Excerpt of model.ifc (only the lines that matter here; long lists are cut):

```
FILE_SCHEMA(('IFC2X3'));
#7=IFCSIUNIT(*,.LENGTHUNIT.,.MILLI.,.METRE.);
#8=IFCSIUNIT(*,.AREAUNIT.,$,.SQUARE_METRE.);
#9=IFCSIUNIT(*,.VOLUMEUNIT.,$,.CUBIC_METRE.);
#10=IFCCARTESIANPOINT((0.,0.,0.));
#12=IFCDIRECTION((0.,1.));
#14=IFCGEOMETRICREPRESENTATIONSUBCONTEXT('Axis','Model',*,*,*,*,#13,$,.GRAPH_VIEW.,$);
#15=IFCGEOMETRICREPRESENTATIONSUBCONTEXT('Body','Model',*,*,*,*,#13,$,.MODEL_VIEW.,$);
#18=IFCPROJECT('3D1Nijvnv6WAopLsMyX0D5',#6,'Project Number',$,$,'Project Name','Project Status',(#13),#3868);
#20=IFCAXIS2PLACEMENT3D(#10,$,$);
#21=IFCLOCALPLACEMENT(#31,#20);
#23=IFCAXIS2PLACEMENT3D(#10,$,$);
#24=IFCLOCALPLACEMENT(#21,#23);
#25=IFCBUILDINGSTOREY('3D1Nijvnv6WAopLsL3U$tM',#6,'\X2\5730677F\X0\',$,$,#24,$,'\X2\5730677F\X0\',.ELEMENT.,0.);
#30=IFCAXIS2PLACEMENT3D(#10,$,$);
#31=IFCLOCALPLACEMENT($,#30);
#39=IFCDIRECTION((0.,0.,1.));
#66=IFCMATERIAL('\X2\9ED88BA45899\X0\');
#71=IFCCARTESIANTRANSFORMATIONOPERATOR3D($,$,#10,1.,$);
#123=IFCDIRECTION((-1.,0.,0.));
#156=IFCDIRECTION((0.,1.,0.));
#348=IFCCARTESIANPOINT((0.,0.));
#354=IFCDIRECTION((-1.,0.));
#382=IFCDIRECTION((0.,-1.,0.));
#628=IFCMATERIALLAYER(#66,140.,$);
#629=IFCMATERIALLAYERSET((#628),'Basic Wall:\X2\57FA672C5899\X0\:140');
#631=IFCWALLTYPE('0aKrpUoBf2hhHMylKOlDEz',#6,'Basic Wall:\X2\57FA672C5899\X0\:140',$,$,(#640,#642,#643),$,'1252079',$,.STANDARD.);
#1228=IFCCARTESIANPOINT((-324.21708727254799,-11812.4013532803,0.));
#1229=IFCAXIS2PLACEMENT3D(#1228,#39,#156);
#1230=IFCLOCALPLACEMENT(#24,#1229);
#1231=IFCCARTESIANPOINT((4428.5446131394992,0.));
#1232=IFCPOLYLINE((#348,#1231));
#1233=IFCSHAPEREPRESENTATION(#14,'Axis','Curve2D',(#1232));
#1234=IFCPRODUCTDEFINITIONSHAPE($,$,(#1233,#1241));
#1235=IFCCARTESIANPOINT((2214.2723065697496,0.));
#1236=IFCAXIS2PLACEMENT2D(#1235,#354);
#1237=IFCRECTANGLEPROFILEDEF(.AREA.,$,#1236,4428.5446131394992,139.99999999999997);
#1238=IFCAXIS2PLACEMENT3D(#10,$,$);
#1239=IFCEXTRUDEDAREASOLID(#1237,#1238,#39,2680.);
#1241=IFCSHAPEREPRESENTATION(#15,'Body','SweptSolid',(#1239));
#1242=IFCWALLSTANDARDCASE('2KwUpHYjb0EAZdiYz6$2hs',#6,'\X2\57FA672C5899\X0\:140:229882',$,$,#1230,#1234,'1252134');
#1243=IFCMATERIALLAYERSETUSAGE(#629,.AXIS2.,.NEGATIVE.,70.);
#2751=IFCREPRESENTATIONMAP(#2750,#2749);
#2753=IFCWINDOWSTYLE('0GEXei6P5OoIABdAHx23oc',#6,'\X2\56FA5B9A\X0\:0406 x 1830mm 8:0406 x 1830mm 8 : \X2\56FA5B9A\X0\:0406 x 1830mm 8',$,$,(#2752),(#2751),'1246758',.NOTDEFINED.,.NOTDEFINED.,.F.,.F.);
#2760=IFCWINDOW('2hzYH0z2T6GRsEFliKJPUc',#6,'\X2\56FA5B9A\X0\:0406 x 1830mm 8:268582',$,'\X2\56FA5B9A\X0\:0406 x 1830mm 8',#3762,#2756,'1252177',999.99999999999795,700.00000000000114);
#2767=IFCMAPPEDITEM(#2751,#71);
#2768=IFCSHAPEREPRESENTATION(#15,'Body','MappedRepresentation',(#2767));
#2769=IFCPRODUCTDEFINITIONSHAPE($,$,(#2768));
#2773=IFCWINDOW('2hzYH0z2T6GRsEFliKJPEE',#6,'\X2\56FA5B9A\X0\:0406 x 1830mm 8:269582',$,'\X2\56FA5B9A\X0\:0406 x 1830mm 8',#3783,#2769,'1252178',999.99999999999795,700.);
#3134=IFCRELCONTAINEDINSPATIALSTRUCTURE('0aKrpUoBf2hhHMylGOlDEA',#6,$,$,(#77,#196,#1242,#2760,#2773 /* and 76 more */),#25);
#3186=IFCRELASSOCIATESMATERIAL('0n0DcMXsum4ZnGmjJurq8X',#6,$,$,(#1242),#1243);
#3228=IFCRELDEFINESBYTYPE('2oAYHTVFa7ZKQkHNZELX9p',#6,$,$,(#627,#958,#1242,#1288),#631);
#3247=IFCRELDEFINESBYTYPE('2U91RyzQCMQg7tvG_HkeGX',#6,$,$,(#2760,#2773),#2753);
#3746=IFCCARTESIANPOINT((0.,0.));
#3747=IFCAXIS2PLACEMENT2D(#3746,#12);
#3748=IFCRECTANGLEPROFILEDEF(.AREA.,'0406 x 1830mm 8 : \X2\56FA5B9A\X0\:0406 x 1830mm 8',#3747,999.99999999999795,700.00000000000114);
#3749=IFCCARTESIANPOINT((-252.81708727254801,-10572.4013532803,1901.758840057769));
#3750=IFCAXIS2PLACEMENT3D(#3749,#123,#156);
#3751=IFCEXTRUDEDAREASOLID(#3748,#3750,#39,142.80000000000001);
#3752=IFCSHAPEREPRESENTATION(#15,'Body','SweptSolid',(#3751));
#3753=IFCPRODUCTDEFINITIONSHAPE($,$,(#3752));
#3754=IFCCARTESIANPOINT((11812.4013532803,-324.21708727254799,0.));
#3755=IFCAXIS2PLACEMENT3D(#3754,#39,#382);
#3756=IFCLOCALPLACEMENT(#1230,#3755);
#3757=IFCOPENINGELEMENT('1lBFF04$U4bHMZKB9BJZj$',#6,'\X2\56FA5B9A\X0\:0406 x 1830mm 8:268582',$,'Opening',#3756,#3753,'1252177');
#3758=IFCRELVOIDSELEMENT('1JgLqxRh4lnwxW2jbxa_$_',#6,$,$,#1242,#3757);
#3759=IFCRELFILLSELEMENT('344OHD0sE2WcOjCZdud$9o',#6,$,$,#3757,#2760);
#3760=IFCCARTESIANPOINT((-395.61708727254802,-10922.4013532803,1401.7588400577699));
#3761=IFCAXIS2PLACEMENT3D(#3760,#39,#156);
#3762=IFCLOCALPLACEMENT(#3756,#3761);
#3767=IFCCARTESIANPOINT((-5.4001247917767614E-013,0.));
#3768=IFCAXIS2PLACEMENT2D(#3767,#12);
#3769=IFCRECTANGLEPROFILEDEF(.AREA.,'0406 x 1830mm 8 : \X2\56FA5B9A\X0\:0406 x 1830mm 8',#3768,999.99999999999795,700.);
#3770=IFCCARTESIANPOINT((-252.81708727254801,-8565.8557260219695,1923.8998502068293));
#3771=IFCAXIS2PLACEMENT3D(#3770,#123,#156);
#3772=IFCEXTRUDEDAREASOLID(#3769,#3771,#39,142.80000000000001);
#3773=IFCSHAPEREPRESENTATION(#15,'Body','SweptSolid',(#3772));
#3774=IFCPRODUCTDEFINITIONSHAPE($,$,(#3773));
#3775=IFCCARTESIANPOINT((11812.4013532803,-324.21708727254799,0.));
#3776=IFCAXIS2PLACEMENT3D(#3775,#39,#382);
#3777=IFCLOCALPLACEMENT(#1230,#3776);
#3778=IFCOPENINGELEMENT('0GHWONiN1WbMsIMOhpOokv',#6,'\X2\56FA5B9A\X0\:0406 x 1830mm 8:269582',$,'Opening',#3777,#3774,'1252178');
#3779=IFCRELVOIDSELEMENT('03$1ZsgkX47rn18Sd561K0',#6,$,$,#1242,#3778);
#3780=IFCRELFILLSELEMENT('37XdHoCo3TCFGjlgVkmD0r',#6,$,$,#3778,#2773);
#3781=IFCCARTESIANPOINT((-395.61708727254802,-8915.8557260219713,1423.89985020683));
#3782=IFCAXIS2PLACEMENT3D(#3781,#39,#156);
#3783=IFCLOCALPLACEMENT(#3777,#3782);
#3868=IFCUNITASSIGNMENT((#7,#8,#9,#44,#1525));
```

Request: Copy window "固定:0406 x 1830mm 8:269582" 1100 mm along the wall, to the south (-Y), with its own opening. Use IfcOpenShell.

```python
import ifcopenshell
import ifcopenshell.api.feature
import ifcopenshell.api.geometry
import ifcopenshell.api.root
import ifcopenshell.geom
import ifcopenshell.util.element
import ifcopenshell.util.placement
import ifcopenshell.util.shape
import ifcopenshell.util.unit

model = ifcopenshell.open("model.ifc")
unit_scale = ifcopenshell.util.unit.calculate_unit_scale(model)
settings = ifcopenshell.geom.settings()


def volume(element):
    """Net volume in cubic metres, openings subtracted."""
    shape = ifcopenshell.geom.create_shape(settings, element)
    return ifcopenshell.util.shape.get_volume(shape.geometry)


def reuse_history(source, copy):
    """copy_class also copies each property set's owner history, people and application; keep the originals."""
    for rel in copy.IsDefinedBy:
        if rel.is_a("IfcRelDefinesByProperties") and (history := rel.RelatingPropertyDefinition.OwnerHistory):
            rel.RelatingPropertyDefinition.OwnerHistory = source.OwnerHistory
            ifcopenshell.util.element.remove_deep2(model, history)


window = model.by_guid("2hzYH0z2T6GRsEFliKJPEE")
opening = window.FillsVoids[0].RelatingOpeningElement
wall = opening.VoidsElements[0].RelatingBuildingElement
before = volume(wall)
shift = ifcopenshell.util.placement.get_local_placement(wall.ObjectPlacement)[:3, 0] * -1.1 / unit_scale

# copy_class copies the void relationship, type, container and properties, but no geometry.
new_opening = ifcopenshell.api.root.copy_class(model, product=opening)
new_opening.Representation = ifcopenshell.util.element.copy_deep(
    model, opening.Representation, exclude=["IfcGeometricRepresentationContext", "IfcRepresentationMap"]
)
new_opening.Name = "固定:0406 x 1830mm 8"
new_opening.Tag = None
new_window = ifcopenshell.api.root.copy_class(model, product=window)
new_window.Representation = ifcopenshell.util.element.copy_deep(
    model, window.Representation, exclude=["IfcGeometricRepresentationContext", "IfcRepresentationMap"]
)
new_window.Name = "固定:0406 x 1830mm 8"
new_window.Tag = None
reuse_history(window, new_window)
fills = ifcopenshell.api.feature.add_filling(model, opening=new_opening, element=new_window)
fills.OwnerHistory = new_window.OwnerHistory  # required in IFC2X3

for old, new in ((opening, new_opening), (window, new_window)):
    matrix = ifcopenshell.util.placement.get_local_placement(old.ObjectPlacement)
    matrix[:3, 3] += shift
    ifcopenshell.api.geometry.edit_object_placement(model, product=new, matrix=matrix, is_si=False)

after = volume(wall)

print(f"wall volume {before:.3f} -> {after:.3f} m3")

model.write("model_edited.ifc")
```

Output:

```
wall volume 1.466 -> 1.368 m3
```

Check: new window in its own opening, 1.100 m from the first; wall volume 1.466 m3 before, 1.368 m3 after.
